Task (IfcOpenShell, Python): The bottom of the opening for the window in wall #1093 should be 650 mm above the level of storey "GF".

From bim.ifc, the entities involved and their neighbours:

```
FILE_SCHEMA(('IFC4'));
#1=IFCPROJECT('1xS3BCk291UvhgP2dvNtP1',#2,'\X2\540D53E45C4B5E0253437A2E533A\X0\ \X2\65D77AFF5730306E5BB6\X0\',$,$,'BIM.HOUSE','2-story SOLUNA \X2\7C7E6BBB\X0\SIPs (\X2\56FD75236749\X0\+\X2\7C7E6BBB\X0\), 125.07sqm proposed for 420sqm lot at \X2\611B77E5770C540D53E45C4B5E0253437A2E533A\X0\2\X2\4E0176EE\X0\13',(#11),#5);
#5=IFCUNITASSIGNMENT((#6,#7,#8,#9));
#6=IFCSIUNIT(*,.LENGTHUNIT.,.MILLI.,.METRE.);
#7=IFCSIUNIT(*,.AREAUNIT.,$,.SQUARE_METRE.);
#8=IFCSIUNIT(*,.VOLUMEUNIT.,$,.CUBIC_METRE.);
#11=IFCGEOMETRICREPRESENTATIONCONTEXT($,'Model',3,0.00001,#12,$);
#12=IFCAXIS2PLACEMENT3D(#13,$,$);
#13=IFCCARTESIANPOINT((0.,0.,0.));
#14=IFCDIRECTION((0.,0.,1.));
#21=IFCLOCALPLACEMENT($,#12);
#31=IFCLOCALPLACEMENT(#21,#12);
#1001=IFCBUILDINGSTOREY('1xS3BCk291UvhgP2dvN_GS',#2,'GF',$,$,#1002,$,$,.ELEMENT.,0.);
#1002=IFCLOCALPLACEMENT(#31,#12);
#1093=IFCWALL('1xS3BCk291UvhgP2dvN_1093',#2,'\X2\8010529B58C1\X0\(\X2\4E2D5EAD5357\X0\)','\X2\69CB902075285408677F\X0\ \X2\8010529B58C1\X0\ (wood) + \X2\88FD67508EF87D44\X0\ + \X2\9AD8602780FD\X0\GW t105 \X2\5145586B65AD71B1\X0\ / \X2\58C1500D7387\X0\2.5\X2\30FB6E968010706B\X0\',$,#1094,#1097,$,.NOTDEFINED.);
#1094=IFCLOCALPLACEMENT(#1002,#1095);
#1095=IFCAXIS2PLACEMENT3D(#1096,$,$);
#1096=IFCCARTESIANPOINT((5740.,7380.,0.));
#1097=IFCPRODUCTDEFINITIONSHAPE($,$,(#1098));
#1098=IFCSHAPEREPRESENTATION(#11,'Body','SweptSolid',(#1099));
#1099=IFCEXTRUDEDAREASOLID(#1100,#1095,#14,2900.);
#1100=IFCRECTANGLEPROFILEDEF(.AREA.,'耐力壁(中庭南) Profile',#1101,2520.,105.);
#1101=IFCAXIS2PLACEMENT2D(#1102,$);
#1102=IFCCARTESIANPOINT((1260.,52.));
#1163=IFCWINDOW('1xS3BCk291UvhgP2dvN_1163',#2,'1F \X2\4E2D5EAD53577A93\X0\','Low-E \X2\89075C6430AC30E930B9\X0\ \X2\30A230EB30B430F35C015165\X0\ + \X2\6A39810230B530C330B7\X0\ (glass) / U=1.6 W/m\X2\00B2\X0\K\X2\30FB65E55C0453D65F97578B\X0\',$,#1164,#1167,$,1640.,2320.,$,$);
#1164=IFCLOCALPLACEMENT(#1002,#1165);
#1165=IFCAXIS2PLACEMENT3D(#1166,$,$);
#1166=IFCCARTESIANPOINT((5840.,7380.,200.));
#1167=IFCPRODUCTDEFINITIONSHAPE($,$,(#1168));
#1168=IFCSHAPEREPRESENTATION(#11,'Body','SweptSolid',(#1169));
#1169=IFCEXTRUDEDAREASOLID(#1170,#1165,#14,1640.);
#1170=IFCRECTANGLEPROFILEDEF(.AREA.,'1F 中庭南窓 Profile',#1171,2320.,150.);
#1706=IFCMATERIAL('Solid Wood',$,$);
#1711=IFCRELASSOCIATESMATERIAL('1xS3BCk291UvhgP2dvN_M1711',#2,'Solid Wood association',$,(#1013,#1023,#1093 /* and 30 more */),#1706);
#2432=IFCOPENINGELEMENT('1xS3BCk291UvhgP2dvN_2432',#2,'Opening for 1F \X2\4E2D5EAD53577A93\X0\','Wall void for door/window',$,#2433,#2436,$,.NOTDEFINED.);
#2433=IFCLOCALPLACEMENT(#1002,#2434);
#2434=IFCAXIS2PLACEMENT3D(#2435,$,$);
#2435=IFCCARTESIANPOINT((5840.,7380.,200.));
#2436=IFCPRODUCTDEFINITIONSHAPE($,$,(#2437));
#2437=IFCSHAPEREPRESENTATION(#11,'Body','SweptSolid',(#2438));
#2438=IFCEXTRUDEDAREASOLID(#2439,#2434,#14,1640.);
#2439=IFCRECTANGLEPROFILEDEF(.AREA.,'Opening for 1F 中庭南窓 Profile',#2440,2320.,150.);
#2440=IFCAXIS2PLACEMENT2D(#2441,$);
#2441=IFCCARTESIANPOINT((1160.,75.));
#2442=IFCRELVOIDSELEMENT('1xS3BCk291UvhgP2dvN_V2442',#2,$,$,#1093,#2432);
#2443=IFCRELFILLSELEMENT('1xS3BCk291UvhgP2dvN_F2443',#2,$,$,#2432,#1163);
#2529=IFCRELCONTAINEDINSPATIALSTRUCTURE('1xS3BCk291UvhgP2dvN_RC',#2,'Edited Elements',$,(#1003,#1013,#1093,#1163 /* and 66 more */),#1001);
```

```python
import numpy as np
import ifcopenshell
import ifcopenshell.api.geometry
import ifcopenshell.geom
import ifcopenshell.util.element
import ifcopenshell.util.placement
import ifcopenshell.util.shape
import ifcopenshell.util.unit

model = ifcopenshell.open("bim.ifc")
unit_scale = ifcopenshell.util.unit.calculate_unit_scale(model)

window = model.by_guid("1xS3BCk291UvhgP2dvN_1163")
opening = window.FillsVoids[0].RelatingOpeningElement
storey = ifcopenshell.util.element.get_container(window, ifc_class="IfcBuildingStorey")
level = ifcopenshell.util.placement.get_local_placement(storey.ObjectPlacement)[2, 3]

# The opening's origin need not be at the sill, so measure its lowest point.
shape = ifcopenshell.geom.create_shape(ifcopenshell.geom.settings(), opening)
bottom = ifcopenshell.util.shape.get_shape_bottom_elevation(shape, shape.geometry) / unit_scale
dz = level + 0.65 / unit_scale - bottom

shift = np.array([0.0, 0.0, dz])
# The window is not placed relative to its opening, so move both.
for product in (opening, window):
    matrix = ifcopenshell.util.placement.get_local_placement(product.ObjectPlacement)
    matrix[:3, 3] += shift
    ifcopenshell.api.geometry.edit_object_placement(model, product=product, matrix=matrix, is_si=False)

print(f"moved by {dz * unit_scale:+.3f} m")

model.write("bim_rev.ifc")
```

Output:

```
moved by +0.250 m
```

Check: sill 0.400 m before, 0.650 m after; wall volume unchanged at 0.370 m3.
